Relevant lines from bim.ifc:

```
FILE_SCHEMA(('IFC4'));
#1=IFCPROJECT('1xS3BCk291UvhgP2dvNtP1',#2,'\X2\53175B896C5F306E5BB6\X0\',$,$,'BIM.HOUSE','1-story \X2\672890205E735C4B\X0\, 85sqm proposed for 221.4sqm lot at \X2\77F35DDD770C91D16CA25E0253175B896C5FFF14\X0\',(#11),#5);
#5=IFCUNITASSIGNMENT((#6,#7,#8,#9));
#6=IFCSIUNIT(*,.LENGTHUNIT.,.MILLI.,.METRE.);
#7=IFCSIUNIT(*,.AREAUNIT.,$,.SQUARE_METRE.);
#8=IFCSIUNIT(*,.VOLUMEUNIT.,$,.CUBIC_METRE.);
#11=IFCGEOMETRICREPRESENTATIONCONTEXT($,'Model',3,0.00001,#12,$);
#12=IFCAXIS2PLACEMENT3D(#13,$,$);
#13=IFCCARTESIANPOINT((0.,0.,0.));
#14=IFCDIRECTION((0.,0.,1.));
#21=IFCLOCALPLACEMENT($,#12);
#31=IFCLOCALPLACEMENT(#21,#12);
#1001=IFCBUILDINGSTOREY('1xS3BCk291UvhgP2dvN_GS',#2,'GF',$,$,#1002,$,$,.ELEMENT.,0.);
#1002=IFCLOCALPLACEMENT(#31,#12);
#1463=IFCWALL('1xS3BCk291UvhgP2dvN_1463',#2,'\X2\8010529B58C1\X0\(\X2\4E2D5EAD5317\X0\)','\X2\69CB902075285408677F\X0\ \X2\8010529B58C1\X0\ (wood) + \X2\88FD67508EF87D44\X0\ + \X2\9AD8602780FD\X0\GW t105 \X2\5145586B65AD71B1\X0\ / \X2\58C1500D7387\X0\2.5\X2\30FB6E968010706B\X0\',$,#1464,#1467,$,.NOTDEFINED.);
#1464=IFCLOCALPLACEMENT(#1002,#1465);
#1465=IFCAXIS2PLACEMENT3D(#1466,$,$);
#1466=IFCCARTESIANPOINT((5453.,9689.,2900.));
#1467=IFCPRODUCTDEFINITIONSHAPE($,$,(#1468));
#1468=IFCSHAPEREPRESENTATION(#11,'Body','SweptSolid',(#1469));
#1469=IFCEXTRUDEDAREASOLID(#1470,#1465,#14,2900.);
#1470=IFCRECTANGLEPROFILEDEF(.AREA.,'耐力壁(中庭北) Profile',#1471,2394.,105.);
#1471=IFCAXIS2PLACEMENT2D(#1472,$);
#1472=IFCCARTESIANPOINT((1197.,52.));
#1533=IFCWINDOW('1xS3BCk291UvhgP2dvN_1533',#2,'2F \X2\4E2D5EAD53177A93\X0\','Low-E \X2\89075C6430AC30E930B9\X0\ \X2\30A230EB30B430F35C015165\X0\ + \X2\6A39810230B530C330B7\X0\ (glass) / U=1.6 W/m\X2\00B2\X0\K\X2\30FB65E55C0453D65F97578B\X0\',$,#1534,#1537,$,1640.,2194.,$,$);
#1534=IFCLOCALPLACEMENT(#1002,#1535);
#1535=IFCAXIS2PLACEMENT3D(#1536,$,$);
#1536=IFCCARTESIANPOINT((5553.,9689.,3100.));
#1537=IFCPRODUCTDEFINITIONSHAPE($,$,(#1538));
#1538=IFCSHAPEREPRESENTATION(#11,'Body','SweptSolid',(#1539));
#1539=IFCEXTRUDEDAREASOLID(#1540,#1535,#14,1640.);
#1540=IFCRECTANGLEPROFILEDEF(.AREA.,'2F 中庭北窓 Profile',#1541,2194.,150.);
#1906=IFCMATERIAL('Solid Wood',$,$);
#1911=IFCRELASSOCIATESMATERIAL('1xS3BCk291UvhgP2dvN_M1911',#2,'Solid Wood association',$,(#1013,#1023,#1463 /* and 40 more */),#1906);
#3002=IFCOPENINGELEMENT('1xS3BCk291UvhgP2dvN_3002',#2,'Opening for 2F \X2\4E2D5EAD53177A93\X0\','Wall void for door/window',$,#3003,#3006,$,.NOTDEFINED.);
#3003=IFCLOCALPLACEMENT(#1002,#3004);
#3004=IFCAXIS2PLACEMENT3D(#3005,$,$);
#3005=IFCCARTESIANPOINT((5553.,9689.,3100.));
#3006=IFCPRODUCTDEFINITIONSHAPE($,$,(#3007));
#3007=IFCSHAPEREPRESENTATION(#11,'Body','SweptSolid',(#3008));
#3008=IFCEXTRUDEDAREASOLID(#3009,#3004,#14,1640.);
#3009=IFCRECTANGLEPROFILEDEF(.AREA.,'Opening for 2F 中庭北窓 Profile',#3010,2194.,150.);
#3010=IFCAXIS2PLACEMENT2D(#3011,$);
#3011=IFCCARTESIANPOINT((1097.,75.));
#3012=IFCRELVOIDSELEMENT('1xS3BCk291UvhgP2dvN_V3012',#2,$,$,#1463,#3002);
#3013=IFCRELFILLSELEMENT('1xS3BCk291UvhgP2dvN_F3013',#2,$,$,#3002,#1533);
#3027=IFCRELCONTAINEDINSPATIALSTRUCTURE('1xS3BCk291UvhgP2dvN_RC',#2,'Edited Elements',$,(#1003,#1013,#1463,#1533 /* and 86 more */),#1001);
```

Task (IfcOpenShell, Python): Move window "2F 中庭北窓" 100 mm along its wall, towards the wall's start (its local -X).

```python
import ifcopenshell
import ifcopenshell.api.geometry
import ifcopenshell.util.placement

model = ifcopenshell.open("bim.ifc")

window = model.by_id(1533)
opening = window.FillsVoids[0].RelatingOpeningElement
wall = opening.VoidsElements[0].RelatingBuildingElement

wall_matrix = ifcopenshell.util.placement.get_local_placement(wall.ObjectPlacement)
shift = wall_matrix[:3, 0] * -100.0
before = ifcopenshell.util.placement.get_local_placement(window.ObjectPlacement)[:3, 3].copy()

# The window is not placed relative to its opening, so move both.
for product in (opening, window):
    matrix = ifcopenshell.util.placement.get_local_placement(product.ObjectPlacement)
    matrix[:3, 3] += shift
    ifcopenshell.api.geometry.edit_object_placement(model, product=product, matrix=matrix, is_si=False)

after = ifcopenshell.util.placement.get_local_placement(window.ObjectPlacement)[:3, 3]
print("window moved by", (after - before).round(3) + 0.0)

model.write("bim_edited.ifc")
```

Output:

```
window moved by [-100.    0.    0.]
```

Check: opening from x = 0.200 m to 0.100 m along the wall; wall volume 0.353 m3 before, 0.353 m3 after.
